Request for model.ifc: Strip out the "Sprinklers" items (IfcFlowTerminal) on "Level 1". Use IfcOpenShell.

First a look at what the model holds.

```python
import ifcopenshell
import ifcopenshell.util.element

model = ifcopenshell.open("model.ifc")
print(model.schema)
storey = next(s for s in model.by_type("IfcBuildingStorey") if s.Name == "Level 1")
terminals = [e for e in ifcopenshell.util.element.get_decomposition(storey) if e.is_a("IfcFlowTerminal")]
seen = {}
for e in terminals:
    element_type = ifcopenshell.util.element.get_type(e)
    name = element_type.Name if element_type not in (None, e) else None
    seen[name] = seen.get(name, 0) + 1
for name, count in sorted(seen.items(), key=str):
    print(count, "x", name)
```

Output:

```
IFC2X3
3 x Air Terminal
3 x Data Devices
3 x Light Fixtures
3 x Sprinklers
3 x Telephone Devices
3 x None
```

```python
import ifcopenshell
import ifcopenshell.api.root
import ifcopenshell.util.element

model = ifcopenshell.open("model.ifc")

storey = next(s for s in model.by_type("IfcBuildingStorey") if s.Name == "Level 1")
terminals = [e for e in ifcopenshell.util.element.get_decomposition(storey) if e.is_a("IfcFlowTerminal")]
targets = [e for e in terminals if (t := ifcopenshell.util.element.get_type(e)) not in (None, e) and t.Name == "Sprinklers"]

for e in targets:
    ifcopenshell.api.root.remove_product(model, product=e)
print(len(targets), "removed")

model.write("model_rev.ifc")
```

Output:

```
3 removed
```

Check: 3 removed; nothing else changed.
